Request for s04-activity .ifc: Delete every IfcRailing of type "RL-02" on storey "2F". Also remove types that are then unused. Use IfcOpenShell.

First a look at what the model holds.

```python
import ifcopenshell
import ifcopenshell.util.element

model = ifcopenshell.open("s04-activity .ifc")
print(model.schema)
storey = next(s for s in model.by_type("IfcBuildingStorey") if s.Name == "2F")
railings = [e for e in ifcopenshell.util.element.get_decomposition(storey) if e.is_a("IfcRailing")]
seen = {}
for e in railings:
    element_type = ifcopenshell.util.element.get_type(e)
    name = element_type.Name if element_type not in (None, e) else None
    seen[name] = seen.get(name, 0) + 1
for name, count in sorted(seen.items(), key=str):
    print(count, "x", name)
```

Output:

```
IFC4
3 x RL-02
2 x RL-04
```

```python
import ifcopenshell
import ifcopenshell.api.root
import ifcopenshell.util.element

model = ifcopenshell.open("s04-activity .ifc")

storey = next(s for s in model.by_type("IfcBuildingStorey") if s.Name == "2F")
railings = [e for e in ifcopenshell.util.element.get_decomposition(storey) if e.is_a("IfcRailing")]
targets = [e for e in railings if (t := ifcopenshell.util.element.get_type(e)) not in (None, e) and t.Name == "RL-02"]
types = {ifcopenshell.util.element.get_type(e) for e in targets} - {None, *targets}

for e in targets:
    ifcopenshell.api.root.remove_product(model, product=e)
print(len(targets), "removed")

unused = [t for t in types if not ifcopenshell.util.element.get_types(t)]
for t in unused:
    ifcopenshell.api.root.remove_product(model, product=t)
print(len(unused), "unused types removed")

model.write("s04-activity _edited.ifc")
```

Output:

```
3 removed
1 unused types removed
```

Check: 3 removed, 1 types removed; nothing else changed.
